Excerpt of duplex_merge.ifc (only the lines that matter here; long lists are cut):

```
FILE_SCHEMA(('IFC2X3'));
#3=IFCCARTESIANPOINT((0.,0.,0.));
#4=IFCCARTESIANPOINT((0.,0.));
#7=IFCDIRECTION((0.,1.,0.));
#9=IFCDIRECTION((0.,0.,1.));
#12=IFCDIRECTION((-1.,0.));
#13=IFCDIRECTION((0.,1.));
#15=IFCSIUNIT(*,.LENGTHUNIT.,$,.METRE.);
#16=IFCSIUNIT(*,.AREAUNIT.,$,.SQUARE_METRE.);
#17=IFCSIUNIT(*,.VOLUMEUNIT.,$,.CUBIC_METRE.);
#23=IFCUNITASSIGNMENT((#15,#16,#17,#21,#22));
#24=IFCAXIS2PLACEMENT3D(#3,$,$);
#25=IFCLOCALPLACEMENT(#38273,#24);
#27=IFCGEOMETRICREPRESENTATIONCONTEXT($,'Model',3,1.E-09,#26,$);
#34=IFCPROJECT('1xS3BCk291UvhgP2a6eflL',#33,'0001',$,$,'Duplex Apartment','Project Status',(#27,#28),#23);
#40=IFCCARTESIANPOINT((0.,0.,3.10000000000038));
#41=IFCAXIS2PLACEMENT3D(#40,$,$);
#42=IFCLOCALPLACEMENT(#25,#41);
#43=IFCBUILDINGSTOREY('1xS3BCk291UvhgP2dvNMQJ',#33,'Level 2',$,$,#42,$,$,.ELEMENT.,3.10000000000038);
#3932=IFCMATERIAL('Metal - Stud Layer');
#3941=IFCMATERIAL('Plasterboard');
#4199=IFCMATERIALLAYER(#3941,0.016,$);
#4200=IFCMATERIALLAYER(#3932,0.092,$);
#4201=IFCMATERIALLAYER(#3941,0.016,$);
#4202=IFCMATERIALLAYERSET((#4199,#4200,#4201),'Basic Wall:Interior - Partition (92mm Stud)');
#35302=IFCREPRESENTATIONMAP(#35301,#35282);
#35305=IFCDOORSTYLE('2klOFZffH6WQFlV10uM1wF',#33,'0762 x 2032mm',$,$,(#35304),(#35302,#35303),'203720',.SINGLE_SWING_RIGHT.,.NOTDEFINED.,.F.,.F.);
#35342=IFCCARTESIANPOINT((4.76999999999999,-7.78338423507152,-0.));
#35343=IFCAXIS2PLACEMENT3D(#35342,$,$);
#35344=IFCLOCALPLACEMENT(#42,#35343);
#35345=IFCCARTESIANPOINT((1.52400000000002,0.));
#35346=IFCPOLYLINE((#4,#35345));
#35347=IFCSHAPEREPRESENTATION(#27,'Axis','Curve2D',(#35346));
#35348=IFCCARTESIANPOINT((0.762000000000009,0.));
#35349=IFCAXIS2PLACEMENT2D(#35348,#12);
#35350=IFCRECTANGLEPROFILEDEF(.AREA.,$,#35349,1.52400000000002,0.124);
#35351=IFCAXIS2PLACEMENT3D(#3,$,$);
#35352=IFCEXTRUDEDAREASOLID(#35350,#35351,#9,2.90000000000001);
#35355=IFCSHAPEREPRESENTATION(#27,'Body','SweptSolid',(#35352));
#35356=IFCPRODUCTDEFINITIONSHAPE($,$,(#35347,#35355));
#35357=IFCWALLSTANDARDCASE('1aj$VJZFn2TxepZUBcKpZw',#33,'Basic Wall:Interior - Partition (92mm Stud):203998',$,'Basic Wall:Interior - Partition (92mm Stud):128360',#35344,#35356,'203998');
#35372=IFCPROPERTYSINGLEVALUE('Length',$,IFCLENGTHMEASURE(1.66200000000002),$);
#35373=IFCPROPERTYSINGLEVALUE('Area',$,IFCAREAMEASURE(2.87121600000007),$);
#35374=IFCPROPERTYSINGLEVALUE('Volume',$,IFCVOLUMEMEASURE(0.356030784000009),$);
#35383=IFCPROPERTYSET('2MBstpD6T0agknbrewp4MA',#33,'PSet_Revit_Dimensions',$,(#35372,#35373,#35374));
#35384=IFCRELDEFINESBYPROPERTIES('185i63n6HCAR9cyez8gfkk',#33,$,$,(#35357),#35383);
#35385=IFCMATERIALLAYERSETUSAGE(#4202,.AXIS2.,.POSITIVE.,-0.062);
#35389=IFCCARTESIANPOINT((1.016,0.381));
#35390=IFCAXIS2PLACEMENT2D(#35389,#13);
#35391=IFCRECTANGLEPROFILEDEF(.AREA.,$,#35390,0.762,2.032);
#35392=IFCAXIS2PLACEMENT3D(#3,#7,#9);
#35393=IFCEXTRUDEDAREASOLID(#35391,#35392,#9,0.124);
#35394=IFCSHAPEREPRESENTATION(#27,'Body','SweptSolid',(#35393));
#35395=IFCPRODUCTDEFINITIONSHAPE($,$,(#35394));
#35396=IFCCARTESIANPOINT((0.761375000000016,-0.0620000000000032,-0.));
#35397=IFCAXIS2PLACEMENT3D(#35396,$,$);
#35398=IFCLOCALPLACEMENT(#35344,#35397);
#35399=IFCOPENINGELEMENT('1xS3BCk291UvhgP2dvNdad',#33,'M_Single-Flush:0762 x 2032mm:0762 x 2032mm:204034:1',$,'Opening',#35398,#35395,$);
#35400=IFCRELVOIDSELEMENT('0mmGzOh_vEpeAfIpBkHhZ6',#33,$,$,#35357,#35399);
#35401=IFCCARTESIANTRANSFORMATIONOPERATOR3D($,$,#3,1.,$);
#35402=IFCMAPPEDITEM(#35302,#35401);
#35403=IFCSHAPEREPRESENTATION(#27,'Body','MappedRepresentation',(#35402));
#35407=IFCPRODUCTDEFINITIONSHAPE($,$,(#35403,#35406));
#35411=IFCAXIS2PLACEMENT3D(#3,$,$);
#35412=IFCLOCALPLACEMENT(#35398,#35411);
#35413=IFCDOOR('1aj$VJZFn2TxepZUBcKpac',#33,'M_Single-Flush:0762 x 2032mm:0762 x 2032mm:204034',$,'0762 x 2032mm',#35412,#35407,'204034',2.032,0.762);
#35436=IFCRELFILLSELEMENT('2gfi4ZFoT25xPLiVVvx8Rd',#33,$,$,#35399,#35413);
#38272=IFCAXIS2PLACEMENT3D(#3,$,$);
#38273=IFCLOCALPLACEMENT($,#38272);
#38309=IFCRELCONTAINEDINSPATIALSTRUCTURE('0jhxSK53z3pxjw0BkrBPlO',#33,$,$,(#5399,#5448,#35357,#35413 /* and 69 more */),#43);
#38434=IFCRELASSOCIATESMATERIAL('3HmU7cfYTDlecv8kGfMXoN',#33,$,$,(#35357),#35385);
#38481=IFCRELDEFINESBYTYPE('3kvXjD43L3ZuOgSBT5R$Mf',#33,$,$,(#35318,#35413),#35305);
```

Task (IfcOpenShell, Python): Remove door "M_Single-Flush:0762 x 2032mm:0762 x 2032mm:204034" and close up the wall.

```python
import ifcopenshell
import ifcopenshell.api.feature
import ifcopenshell.api.pset
import ifcopenshell.api.root
import ifcopenshell.geom
import ifcopenshell.util.element
import ifcopenshell.util.shape
import ifcopenshell.util.unit

model = ifcopenshell.open("duplex_merge.ifc")
area_scale = ifcopenshell.util.unit.calculate_unit_scale(model, "AREAUNIT")
volume_scale = ifcopenshell.util.unit.calculate_unit_scale(model, "VOLUMEUNIT")
settings = ifcopenshell.geom.settings()


def volume(element):
    """Net volume in cubic metres, openings subtracted."""
    shape = ifcopenshell.geom.create_shape(settings, element)
    return ifcopenshell.util.shape.get_volume(shape.geometry)


door = model.by_guid("1aj$VJZFn2TxepZUBcKpac")
opening = door.FillsVoids[0].RelatingOpeningElement
wall = opening.VoidsElements[0].RelatingBuildingElement
before = volume(wall)

ifcopenshell.api.root.remove_product(model, product=door)
ifcopenshell.api.feature.remove_feature(model, feature=opening)

after = volume(wall)
thickness = 0.124  # wall thickness in metres

# Update the wall's stored quantities.
pset = model.by_id(ifcopenshell.util.element.get_pset(wall, "PSet_Revit_Dimensions", should_inherit=False)["id"])
ifcopenshell.api.pset.edit_pset(model, pset=pset, properties={
    "Area": model.create_entity("IfcAreaMeasure", after / thickness / area_scale),
    "Volume": model.create_entity("IfcVolumeMeasure", after / volume_scale),
})

print(f"wall volume {before:.3f} -> {after:.3f} m3")

model.write("duplex_merge_updated.ifc")
```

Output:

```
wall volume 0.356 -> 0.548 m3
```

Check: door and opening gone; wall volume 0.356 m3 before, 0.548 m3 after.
